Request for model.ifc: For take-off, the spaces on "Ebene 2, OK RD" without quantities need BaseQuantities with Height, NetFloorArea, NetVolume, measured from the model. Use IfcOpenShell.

First a look at what the model holds.

```python
import ifcopenshell
import ifcopenshell.util.element
import ifcopenshell.util.unit

model = ifcopenshell.open("model.ifc")
print(model.schema)
for unit_type in ("LENGTHUNIT", "AREAUNIT", "VOLUMEUNIT"):
    print(unit_type, ifcopenshell.util.unit.calculate_unit_scale(model, unit_type))
storey = next(s for s in model.by_type("IfcBuildingStorey") if s.Name == "Ebene 2, OK RD")
spaces = [e for e in ifcopenshell.util.element.get_decomposition(storey) if e.is_a("IfcSpace")]
for e in sorted(spaces, key=lambda e: e.id()):
    print(e.id(), e.is_a(), e.Name, list(ifcopenshell.util.element.get_psets(e, qtos_only=True)), sep=" | ")
```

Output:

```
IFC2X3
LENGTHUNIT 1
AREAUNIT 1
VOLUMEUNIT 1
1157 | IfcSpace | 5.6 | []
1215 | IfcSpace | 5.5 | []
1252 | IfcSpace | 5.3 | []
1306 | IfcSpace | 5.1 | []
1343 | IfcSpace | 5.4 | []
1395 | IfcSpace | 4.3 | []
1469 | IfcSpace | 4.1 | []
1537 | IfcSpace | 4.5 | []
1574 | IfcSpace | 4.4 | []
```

```python
import ifcopenshell
import ifcopenshell.api.pset
import ifcopenshell.geom
import ifcopenshell.util.element
import ifcopenshell.util.shape
import ifcopenshell.util.unit

model = ifcopenshell.open("model.ifc")
unit_scale = ifcopenshell.util.unit.calculate_unit_scale(model)
area_scale = ifcopenshell.util.unit.calculate_unit_scale(model, "AREAUNIT")
volume_scale = ifcopenshell.util.unit.calculate_unit_scale(model, "VOLUMEUNIT")
settings = ifcopenshell.geom.settings()

storey = next(s for s in model.by_type("IfcBuildingStorey") if s.Name == "Ebene 2, OK RD")
spaces = [e for e in ifcopenshell.util.element.get_decomposition(storey) if e.is_a("IfcSpace")]

for e in sorted(spaces, key=lambda e: e.id()):
    if ifcopenshell.util.element.get_psets(e, qtos_only=True, should_inherit=False):
        continue
    # Geometry comes back in metres, in the element's own axes.
    shape = ifcopenshell.geom.create_shape(settings, e)
    values = {
        "Height": ifcopenshell.util.shape.get_z(shape.geometry) / unit_scale,
        "NetFloorArea": ifcopenshell.util.shape.get_footprint_area(shape.geometry) / area_scale,
        "NetVolume": ifcopenshell.util.shape.get_volume(shape.geometry) / volume_scale,
    }
    qto = ifcopenshell.api.pset.add_qto(model, product=e, name="BaseQuantities")
    ifcopenshell.api.pset.edit_qto(model, qto=qto, properties=values)
    print(e.id(), {k: round(v, 3) for k, v in values.items()})

model.write("model_rev.ifc")
```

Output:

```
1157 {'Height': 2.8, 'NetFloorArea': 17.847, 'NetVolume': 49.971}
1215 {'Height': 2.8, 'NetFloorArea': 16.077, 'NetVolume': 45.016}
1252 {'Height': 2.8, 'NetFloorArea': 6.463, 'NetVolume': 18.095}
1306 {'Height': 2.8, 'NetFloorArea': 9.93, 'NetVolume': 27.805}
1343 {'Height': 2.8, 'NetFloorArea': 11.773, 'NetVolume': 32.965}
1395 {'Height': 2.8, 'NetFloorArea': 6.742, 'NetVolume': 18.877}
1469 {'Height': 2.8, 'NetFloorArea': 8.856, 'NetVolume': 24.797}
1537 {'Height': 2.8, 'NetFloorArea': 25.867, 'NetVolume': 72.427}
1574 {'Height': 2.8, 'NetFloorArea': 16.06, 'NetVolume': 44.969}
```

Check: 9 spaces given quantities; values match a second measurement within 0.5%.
